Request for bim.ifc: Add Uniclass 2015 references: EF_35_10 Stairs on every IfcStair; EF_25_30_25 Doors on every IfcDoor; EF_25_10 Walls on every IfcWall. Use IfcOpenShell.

First a look at what the model holds.

```python
import ifcopenshell

model = ifcopenshell.open("bim.ifc")
print(model.schema)
print("classifications:", [c.Name for c in model.by_type("IfcClassification")])
for ifc_class in ("IfcDoor", "IfcRoof", "IfcStair", "IfcWall", "IfcWindow"):
    print(ifc_class, len(model.by_type(ifc_class)))
```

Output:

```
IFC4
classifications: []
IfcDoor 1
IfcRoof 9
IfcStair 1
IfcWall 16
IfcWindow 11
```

```python
import ifcopenshell
import ifcopenshell.api.classification

model = ifcopenshell.open("bim.ifc")

system = ifcopenshell.api.classification.add_classification(model, classification="Uniclass 2015")

codes = {
    "IfcStair": ("EF_35_10", "Stairs"),
    "IfcDoor": ("EF_25_30_25", "Doors"),
    "IfcWall": ("EF_25_10", "Walls"),
}
for ifc_class, (code, name) in codes.items():
    products = model.by_type(ifc_class)
    ifcopenshell.api.classification.add_reference(
        model, products=products, classification=system, identification=code, name=name
    )
    print(code, len(products))

model.write("bim_v2.ifc")
```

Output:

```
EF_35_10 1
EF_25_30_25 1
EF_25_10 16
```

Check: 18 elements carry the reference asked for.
